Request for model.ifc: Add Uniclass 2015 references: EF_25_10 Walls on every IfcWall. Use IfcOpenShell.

First a look at what the model holds.

```python
import ifcopenshell

model = ifcopenshell.open("model.ifc")
print(model.schema)
print("classifications:", [c.Name for c in model.by_type("IfcClassification")])
for ifc_class in ("IfcDoor", "IfcRoof", "IfcStair", "IfcWall", "IfcWindow"):
    print(ifc_class, len(model.by_type(ifc_class)))
```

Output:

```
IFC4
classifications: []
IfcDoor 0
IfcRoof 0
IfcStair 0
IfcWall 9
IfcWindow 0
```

```python
import ifcopenshell
import ifcopenshell.api.classification

model = ifcopenshell.open("model.ifc")

system = ifcopenshell.api.classification.add_classification(model, classification="Uniclass 2015")

codes = {
    "IfcWall": ("EF_25_10", "Walls"),
}
for ifc_class, (code, name) in codes.items():
    products = model.by_type(ifc_class)
    ifcopenshell.api.classification.add_reference(
        model, products=products, classification=system, identification=code, name=name
    )
    print(code, len(products))

model.write("model_updated.ifc")
```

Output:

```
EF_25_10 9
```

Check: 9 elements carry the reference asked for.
